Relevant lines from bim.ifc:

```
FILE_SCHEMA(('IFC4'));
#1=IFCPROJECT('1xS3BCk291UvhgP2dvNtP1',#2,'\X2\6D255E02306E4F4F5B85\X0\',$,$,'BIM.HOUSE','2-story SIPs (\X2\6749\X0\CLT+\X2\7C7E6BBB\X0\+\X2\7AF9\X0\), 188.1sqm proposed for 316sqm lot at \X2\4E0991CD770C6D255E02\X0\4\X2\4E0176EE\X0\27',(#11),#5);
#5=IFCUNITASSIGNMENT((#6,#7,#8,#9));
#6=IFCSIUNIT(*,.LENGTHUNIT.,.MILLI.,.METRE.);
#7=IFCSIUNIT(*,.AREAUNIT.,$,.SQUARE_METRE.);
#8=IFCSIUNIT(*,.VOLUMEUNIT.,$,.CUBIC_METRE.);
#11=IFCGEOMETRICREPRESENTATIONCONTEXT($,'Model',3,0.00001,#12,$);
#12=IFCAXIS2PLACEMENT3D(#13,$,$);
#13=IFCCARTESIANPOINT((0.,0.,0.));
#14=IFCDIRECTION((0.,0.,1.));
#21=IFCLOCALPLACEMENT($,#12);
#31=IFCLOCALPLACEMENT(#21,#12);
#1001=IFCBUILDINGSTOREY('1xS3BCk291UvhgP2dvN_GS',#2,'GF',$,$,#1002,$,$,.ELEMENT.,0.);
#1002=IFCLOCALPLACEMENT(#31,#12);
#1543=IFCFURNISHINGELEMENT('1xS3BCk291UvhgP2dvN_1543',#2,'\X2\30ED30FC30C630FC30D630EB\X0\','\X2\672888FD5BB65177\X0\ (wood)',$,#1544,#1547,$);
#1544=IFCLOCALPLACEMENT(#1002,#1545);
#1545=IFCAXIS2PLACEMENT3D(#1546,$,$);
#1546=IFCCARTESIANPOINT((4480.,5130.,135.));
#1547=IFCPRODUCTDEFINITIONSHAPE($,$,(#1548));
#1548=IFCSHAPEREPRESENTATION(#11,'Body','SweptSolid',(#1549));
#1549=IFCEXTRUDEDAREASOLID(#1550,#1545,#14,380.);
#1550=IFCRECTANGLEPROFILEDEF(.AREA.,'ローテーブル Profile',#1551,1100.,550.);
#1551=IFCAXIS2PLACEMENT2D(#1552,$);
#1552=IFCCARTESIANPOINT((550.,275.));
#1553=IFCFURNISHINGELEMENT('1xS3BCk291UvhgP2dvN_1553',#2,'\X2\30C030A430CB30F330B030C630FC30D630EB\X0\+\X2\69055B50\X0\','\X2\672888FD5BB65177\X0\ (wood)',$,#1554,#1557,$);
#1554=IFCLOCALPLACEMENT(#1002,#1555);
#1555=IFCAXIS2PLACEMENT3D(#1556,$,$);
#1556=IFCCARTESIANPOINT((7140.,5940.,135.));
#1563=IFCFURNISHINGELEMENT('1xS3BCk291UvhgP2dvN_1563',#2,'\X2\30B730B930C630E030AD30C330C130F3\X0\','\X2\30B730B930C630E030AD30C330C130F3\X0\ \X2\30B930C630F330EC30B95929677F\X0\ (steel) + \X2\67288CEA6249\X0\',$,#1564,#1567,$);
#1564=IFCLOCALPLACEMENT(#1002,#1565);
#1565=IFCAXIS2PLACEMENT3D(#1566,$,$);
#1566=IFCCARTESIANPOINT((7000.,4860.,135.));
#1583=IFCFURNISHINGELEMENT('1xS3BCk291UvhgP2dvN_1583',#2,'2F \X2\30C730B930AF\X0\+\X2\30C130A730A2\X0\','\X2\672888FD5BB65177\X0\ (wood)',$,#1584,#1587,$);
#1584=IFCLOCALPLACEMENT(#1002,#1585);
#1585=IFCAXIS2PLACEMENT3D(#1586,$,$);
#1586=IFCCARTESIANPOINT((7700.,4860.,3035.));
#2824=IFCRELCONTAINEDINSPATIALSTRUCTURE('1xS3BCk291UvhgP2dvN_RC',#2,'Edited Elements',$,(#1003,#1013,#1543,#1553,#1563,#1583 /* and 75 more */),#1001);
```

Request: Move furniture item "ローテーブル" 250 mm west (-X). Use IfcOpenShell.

```python
import ifcopenshell
import ifcopenshell.api.geometry
import ifcopenshell.util.placement

model = ifcopenshell.open("bim.ifc")

item = model.by_guid("1xS3BCk291UvhgP2dvN_1543")
matrix = ifcopenshell.util.placement.get_local_placement(item.ObjectPlacement)
matrix[0, 3] -= 250.0
ifcopenshell.api.geometry.edit_object_placement(model, product=item, matrix=matrix, is_si=False)

print(ifcopenshell.util.placement.get_local_placement(item.ObjectPlacement).round(3) + 0.0)

model.write("bim_updated.ifc")
```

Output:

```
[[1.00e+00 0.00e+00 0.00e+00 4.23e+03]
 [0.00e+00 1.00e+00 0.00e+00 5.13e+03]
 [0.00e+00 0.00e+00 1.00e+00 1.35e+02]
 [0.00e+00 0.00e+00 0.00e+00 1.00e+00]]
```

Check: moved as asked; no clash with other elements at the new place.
